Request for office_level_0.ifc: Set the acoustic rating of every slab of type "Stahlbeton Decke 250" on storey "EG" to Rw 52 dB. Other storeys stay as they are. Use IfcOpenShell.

First a look at what the model holds.

```python
import ifcopenshell
import ifcopenshell.util.element

model = ifcopenshell.open("office_level_0.ifc")
print(model.schema)
storey = next(s for s in model.by_type("IfcBuildingStorey") if s.Name == "EG")
slabs = [e for e in ifcopenshell.util.element.get_decomposition(storey) if e.is_a("IfcSlab")]
seen = {}
for e in slabs:
    element_type = ifcopenshell.util.element.get_type(e)
    key = (element_type.Name if element_type != e and element_type else None, ifcopenshell.util.element.get_pset(e, "Pset_SlabCommon", "AcousticRating"))
    seen[key] = seen.get(key, 0) + 1
for (name, value), count in sorted(seen.items(), key=str):
    print(count, "x", name, "|", value)
```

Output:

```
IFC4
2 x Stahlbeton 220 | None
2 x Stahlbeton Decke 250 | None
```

```python
import ifcopenshell
import ifcopenshell.api.pset
import ifcopenshell.util.element

model = ifcopenshell.open("office_level_0.ifc")

storey = next(s for s in model.by_type("IfcBuildingStorey") if s.Name == "EG")
slabs = [e for e in ifcopenshell.util.element.get_decomposition(storey) if e.is_a("IfcSlab")]

count = 0
for e in slabs:
    element_type = ifcopenshell.util.element.get_type(e)
    if element_type in (None, e) or element_type.Name != "Stahlbeton Decke 250":
        continue
    # add_pset returns the element's existing set when there is one.
    pset = ifcopenshell.api.pset.add_pset(model, product=e, name="Pset_SlabCommon")
    ifcopenshell.api.pset.edit_pset(model, pset=pset, properties={"AcousticRating": "Rw 52 dB"})
    count += 1

print(count, "slabs updated")

model.write("office_level_0_edited.ifc")
```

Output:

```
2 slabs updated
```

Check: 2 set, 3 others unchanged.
